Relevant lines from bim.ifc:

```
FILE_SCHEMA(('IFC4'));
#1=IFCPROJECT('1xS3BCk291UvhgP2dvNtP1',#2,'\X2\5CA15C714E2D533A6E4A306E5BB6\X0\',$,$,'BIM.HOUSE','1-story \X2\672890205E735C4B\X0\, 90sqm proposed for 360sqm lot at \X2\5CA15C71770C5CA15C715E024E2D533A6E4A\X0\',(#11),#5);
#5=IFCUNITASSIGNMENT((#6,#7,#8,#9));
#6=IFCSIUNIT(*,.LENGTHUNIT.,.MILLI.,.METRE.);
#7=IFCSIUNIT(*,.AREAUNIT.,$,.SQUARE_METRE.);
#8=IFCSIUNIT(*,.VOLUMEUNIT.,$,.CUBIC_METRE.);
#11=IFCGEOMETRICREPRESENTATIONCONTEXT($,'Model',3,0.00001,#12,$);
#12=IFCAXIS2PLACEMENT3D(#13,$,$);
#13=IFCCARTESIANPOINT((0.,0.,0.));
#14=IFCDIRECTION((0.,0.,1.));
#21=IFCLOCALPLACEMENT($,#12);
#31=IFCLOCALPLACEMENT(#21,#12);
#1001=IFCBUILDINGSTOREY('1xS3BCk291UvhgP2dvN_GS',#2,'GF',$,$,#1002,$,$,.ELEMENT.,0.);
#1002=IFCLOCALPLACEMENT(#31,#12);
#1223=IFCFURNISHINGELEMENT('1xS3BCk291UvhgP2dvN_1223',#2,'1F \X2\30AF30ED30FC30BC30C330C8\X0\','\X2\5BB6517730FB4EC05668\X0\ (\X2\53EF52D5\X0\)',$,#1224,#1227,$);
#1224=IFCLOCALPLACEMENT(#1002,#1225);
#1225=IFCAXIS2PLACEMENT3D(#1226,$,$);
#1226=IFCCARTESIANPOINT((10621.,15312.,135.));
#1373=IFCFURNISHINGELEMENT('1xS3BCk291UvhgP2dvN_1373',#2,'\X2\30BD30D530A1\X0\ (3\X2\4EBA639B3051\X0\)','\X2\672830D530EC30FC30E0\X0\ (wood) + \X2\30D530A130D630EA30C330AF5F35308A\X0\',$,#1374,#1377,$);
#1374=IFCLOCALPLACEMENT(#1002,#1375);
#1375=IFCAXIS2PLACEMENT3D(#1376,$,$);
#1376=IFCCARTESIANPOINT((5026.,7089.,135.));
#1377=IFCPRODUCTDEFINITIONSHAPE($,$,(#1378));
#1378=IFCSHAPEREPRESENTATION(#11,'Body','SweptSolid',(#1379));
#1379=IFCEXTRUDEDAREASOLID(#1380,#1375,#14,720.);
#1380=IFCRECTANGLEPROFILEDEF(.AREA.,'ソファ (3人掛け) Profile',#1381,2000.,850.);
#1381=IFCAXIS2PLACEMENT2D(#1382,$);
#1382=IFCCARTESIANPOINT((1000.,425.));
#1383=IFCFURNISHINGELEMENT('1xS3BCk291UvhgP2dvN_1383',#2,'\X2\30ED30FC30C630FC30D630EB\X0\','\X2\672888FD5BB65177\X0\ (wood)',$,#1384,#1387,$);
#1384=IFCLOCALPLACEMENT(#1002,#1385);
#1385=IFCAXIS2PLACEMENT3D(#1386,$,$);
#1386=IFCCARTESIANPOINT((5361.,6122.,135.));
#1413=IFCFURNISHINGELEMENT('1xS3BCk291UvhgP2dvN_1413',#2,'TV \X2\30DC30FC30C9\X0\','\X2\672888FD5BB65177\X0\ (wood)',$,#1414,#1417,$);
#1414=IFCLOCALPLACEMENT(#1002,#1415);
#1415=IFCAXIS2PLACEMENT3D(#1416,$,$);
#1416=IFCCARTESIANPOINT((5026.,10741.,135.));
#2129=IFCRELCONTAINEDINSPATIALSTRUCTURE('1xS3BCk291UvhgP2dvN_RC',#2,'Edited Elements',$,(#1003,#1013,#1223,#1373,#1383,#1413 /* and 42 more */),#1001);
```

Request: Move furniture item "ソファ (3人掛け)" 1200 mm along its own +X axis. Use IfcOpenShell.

```python
import ifcopenshell
import ifcopenshell.api.geometry
import ifcopenshell.util.placement
import ifcopenshell.util.unit

model = ifcopenshell.open("bim.ifc")
unit_scale = ifcopenshell.util.unit.calculate_unit_scale(model)

item = model.by_id(1373)
matrix = ifcopenshell.util.placement.get_local_placement(item.ObjectPlacement)
matrix[:3, 3] += matrix[:3, 0] * 1.2 / unit_scale
ifcopenshell.api.geometry.edit_object_placement(model, product=item, matrix=matrix, is_si=False)

print(ifcopenshell.util.placement.get_local_placement(item.ObjectPlacement).round(3) + 0.0)

model.write("bim_edited.ifc")
```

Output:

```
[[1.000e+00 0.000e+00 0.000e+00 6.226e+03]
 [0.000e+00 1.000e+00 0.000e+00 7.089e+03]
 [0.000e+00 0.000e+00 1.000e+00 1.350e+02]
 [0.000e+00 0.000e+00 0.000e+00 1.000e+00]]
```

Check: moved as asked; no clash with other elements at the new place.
